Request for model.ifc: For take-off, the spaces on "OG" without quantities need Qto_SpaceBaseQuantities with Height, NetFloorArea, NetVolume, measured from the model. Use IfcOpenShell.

First a look at what the model holds.

```python
import ifcopenshell
import ifcopenshell.util.element
import ifcopenshell.util.unit

model = ifcopenshell.open("model.ifc")
print(model.schema)
for unit_type in ("LENGTHUNIT", "AREAUNIT", "VOLUMEUNIT"):
    print(unit_type, ifcopenshell.util.unit.calculate_unit_scale(model, unit_type))
storey = next(s for s in model.by_type("IfcBuildingStorey") if s.Name == "OG")
spaces = [e for e in ifcopenshell.util.element.get_decomposition(storey) if e.is_a("IfcSpace")]
for e in sorted(spaces, key=lambda e: e.id()):
    print(e.id(), e.is_a(), e.Name, list(ifcopenshell.util.element.get_psets(e, qtos_only=True)), sep=" | ")
```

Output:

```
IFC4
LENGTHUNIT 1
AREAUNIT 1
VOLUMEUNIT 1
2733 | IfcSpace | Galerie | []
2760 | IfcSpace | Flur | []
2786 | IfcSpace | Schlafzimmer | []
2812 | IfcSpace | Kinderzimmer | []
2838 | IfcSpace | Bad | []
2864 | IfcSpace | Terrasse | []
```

```python
import ifcopenshell
import ifcopenshell.api.pset
import ifcopenshell.geom
import ifcopenshell.util.element
import ifcopenshell.util.shape
import ifcopenshell.util.unit

model = ifcopenshell.open("model.ifc")
unit_scale = ifcopenshell.util.unit.calculate_unit_scale(model)
area_scale = ifcopenshell.util.unit.calculate_unit_scale(model, "AREAUNIT")
volume_scale = ifcopenshell.util.unit.calculate_unit_scale(model, "VOLUMEUNIT")
settings = ifcopenshell.geom.settings()

storey = next(s for s in model.by_type("IfcBuildingStorey") if s.Name == "OG")
spaces = [e for e in ifcopenshell.util.element.get_decomposition(storey) if e.is_a("IfcSpace")]

for e in sorted(spaces, key=lambda e: e.id()):
    if ifcopenshell.util.element.get_psets(e, qtos_only=True, should_inherit=False):
        continue
    # Geometry comes back in metres, in the element's own axes.
    shape = ifcopenshell.geom.create_shape(settings, e)
    values = {
        "Height": ifcopenshell.util.shape.get_z(shape.geometry) / unit_scale,
        "NetFloorArea": ifcopenshell.util.shape.get_footprint_area(shape.geometry) / area_scale,
        "NetVolume": ifcopenshell.util.shape.get_volume(shape.geometry) / volume_scale,
    }
    qto = ifcopenshell.api.pset.add_qto(model, product=e, name="Qto_SpaceBaseQuantities")
    ifcopenshell.api.pset.edit_qto(model, qto=qto, properties=values)
    print(e.id(), {k: round(v, 3) for k, v in values.items()})

model.write("model-out.ifc")
```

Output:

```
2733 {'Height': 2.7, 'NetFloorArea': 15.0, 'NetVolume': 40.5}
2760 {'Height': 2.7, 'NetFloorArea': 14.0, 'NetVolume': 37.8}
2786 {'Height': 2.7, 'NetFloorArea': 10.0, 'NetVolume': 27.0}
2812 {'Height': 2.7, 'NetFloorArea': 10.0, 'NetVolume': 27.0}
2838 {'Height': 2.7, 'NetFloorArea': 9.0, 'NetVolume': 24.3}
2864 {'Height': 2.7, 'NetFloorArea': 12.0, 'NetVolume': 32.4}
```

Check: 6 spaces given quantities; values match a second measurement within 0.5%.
